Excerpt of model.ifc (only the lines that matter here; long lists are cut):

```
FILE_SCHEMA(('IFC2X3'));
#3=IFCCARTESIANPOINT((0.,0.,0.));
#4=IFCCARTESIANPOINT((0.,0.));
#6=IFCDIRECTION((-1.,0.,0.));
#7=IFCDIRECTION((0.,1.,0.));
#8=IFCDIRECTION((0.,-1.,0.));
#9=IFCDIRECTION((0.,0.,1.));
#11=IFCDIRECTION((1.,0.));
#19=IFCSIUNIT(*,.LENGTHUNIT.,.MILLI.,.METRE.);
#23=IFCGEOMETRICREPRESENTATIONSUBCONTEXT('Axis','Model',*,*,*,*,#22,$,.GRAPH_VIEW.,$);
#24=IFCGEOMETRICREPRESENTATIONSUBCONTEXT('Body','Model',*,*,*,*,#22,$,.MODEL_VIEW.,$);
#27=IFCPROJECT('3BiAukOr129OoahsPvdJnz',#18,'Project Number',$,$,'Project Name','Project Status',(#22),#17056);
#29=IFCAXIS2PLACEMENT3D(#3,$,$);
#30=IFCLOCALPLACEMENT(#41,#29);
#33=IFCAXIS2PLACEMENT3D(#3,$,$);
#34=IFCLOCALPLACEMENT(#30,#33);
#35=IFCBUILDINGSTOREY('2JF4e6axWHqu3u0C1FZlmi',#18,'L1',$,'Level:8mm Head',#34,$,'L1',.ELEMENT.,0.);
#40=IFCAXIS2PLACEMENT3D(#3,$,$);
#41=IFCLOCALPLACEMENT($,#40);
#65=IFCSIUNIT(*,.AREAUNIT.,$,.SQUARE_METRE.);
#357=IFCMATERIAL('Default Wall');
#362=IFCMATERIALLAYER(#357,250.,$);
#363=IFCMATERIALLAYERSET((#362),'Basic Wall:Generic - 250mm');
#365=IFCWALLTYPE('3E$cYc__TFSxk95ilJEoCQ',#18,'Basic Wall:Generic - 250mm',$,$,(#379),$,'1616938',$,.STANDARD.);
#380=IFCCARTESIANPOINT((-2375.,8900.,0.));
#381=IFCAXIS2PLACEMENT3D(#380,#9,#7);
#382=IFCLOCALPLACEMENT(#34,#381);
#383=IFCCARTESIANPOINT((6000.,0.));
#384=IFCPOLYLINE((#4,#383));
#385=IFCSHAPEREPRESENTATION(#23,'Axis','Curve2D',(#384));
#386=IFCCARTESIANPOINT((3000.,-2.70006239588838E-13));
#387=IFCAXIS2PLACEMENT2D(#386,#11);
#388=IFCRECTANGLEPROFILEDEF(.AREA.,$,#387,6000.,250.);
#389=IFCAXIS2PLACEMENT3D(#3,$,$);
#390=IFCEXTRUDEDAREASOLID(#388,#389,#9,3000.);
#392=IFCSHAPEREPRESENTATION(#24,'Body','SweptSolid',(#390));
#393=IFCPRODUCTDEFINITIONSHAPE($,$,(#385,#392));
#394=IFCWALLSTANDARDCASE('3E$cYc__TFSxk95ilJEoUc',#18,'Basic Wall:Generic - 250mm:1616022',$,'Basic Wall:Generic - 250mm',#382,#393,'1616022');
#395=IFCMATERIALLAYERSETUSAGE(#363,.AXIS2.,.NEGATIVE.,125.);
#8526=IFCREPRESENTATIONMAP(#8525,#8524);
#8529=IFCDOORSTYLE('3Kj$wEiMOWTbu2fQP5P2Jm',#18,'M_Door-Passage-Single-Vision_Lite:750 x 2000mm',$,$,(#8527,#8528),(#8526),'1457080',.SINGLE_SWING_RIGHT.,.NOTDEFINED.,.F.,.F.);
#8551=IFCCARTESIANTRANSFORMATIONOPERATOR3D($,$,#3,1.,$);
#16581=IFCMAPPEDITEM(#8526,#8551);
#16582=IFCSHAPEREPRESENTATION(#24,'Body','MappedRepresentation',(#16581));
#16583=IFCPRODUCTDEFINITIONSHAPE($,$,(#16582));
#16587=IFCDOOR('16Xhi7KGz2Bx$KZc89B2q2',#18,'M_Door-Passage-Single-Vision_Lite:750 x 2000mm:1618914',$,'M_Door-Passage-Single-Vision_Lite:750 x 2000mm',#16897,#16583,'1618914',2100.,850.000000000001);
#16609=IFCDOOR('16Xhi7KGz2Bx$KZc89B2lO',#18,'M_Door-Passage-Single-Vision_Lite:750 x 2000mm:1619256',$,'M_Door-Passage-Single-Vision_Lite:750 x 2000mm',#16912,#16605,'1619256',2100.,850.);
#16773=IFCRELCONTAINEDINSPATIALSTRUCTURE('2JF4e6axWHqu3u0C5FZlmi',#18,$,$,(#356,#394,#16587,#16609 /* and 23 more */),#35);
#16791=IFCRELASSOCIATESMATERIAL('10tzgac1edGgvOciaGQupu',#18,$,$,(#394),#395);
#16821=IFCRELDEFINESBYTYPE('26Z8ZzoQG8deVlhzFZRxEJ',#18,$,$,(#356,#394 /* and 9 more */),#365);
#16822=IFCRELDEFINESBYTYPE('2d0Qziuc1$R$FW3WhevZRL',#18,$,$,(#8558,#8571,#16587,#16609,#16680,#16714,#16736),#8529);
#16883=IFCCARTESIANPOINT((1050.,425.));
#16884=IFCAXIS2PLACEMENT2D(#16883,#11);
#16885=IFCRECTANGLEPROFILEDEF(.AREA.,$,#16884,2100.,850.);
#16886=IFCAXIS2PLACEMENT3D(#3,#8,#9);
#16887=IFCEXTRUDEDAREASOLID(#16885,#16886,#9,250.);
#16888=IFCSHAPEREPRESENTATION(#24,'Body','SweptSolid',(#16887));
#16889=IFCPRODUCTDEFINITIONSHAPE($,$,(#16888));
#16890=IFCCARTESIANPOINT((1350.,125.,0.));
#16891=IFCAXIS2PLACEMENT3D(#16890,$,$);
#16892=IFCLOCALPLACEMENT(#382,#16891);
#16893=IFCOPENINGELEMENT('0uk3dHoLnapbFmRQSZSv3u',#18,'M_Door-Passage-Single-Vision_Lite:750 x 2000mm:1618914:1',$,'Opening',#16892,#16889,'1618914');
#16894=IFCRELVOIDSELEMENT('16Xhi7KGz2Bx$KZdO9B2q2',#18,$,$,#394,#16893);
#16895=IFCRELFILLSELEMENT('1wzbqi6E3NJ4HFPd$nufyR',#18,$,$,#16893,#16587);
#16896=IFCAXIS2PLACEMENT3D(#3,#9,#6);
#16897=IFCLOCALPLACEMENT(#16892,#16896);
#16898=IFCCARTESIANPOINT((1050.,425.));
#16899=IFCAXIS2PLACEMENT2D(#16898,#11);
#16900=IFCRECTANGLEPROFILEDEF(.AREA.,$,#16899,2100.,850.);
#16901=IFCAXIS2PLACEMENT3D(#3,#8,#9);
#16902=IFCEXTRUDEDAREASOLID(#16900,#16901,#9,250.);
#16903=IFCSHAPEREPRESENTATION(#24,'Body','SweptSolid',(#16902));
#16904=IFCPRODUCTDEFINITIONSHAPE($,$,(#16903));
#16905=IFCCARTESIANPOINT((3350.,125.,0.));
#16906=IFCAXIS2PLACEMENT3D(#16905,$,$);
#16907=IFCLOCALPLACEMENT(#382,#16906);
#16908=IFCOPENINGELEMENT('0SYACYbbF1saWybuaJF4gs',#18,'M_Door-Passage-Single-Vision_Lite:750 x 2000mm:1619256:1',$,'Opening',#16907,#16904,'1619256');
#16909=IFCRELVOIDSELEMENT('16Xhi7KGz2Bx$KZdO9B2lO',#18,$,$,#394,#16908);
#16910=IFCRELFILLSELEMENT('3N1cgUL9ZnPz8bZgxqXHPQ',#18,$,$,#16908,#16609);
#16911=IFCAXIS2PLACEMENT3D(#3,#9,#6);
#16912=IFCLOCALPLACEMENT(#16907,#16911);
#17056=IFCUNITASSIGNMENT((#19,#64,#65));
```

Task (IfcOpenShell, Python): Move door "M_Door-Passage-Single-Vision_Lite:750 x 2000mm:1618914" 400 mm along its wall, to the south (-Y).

```python
import ifcopenshell
import ifcopenshell.api.geometry
import ifcopenshell.util.placement
import ifcopenshell.util.unit

model = ifcopenshell.open("model.ifc")
unit_scale = ifcopenshell.util.unit.calculate_unit_scale(model)

door = model.by_guid("16Xhi7KGz2Bx$KZc89B2q2")
opening = door.FillsVoids[0].RelatingOpeningElement
wall = opening.VoidsElements[0].RelatingBuildingElement

wall_matrix = ifcopenshell.util.placement.get_local_placement(wall.ObjectPlacement)
shift = wall_matrix[:3, 0] * -0.4 / unit_scale
before = ifcopenshell.util.placement.get_local_placement(door.ObjectPlacement)[:3, 3].copy()

# The door is placed relative to its opening, so it follows when the opening moves.
matrix = ifcopenshell.util.placement.get_local_placement(opening.ObjectPlacement)
matrix[:3, 3] += shift
ifcopenshell.api.geometry.edit_object_placement(
    model, product=opening, matrix=matrix, is_si=False, should_transform_children=True
)

after = ifcopenshell.util.placement.get_local_placement(door.ObjectPlacement)[:3, 3]
print("door moved by", (after - before).round(3) + 0.0)

model.write("model_v2.ifc")
```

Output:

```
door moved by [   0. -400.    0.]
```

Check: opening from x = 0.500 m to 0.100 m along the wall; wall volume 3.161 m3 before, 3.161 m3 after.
